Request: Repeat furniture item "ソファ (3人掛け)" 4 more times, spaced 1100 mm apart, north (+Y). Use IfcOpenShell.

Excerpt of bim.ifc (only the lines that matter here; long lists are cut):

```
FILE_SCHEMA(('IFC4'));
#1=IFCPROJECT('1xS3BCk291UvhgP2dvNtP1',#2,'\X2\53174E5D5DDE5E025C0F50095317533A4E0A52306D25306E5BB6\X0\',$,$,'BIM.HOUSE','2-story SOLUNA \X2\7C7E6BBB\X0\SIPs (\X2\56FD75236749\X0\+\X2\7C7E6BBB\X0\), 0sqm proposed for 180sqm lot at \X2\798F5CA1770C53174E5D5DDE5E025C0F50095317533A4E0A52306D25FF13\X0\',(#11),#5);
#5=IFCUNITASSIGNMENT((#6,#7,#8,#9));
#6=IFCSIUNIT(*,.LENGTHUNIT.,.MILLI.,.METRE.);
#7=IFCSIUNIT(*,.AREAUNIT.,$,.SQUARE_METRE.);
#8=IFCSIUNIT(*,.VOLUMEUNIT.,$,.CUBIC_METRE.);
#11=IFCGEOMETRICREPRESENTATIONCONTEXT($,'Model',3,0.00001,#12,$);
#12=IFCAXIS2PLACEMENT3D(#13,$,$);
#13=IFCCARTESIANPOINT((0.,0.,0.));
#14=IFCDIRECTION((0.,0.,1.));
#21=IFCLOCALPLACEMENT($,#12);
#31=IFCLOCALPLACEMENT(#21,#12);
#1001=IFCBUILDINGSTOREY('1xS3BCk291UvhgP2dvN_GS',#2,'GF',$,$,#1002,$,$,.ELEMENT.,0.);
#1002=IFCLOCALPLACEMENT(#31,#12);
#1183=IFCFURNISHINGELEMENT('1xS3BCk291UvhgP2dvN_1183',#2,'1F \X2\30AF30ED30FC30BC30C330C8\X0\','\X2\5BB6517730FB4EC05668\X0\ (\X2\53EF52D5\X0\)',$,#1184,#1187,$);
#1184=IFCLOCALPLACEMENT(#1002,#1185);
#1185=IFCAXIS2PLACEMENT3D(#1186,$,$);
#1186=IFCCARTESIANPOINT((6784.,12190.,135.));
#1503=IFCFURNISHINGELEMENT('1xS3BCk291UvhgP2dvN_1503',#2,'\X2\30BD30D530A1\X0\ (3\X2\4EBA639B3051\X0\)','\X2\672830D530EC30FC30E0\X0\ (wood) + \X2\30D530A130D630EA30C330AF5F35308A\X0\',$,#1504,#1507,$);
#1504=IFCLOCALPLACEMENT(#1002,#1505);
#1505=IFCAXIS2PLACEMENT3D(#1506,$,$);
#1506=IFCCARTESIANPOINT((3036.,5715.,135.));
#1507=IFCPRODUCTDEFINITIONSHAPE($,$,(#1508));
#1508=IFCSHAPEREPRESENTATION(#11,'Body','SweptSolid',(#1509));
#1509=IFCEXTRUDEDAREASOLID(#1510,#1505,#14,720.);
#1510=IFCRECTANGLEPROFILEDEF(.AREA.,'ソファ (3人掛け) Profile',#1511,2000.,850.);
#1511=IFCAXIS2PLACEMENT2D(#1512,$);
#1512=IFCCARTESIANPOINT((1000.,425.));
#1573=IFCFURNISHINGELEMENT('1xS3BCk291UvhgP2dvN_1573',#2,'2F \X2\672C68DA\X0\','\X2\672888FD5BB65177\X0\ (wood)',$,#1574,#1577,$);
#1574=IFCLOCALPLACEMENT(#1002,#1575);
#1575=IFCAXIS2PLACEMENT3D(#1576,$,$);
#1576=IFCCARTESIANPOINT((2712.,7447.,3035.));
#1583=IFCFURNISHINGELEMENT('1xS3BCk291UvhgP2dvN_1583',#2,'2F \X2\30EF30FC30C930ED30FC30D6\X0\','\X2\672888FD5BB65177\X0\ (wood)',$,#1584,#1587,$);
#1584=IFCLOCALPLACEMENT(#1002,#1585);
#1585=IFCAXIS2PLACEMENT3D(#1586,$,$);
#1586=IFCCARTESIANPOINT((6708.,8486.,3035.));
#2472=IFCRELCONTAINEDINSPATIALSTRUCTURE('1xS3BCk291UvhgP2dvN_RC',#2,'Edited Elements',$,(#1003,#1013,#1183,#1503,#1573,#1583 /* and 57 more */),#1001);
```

```python
import numpy as np
import ifcopenshell
import ifcopenshell.api.geometry
import ifcopenshell.api.root
import ifcopenshell.util.element
import ifcopenshell.util.placement
import ifcopenshell.util.unit

model = ifcopenshell.open("bim.ifc")
unit_scale = ifcopenshell.util.unit.calculate_unit_scale(model)


def reuse_history(source, copy):
    """copy_class also copies each property set's owner history, people and application; keep the originals."""
    for rel in copy.IsDefinedBy:
        if rel.is_a("IfcRelDefinesByProperties") and (history := rel.RelatingPropertyDefinition.OwnerHistory):
            rel.RelatingPropertyDefinition.OwnerHistory = source.OwnerHistory
            ifcopenshell.util.element.remove_deep2(model, history)


source = model.by_guid("1xS3BCk291UvhgP2dvN_1503")
base = ifcopenshell.util.placement.get_local_placement(source.ObjectPlacement)
step = np.array([0.0, 1.0, 0.0]) * 1.1 / unit_scale

for i in range(1, 5):
    copy = ifcopenshell.api.root.copy_class(model, product=source)
    copy.Representation = ifcopenshell.util.element.copy_deep(
        model, source.Representation, exclude=["IfcGeometricRepresentationContext", "IfcRepresentationMap"]
    )
    reuse_history(source, copy)
    matrix = base.copy()
    matrix[:3, 3] += i * step
    print("added at", matrix[:3, 3].round(3) + 0.0)
    ifcopenshell.api.geometry.edit_object_placement(model, product=copy, matrix=matrix, is_si=False)

model.write("bim_edited.ifc")
```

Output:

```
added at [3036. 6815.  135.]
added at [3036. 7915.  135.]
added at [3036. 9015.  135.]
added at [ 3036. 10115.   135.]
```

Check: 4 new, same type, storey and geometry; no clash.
